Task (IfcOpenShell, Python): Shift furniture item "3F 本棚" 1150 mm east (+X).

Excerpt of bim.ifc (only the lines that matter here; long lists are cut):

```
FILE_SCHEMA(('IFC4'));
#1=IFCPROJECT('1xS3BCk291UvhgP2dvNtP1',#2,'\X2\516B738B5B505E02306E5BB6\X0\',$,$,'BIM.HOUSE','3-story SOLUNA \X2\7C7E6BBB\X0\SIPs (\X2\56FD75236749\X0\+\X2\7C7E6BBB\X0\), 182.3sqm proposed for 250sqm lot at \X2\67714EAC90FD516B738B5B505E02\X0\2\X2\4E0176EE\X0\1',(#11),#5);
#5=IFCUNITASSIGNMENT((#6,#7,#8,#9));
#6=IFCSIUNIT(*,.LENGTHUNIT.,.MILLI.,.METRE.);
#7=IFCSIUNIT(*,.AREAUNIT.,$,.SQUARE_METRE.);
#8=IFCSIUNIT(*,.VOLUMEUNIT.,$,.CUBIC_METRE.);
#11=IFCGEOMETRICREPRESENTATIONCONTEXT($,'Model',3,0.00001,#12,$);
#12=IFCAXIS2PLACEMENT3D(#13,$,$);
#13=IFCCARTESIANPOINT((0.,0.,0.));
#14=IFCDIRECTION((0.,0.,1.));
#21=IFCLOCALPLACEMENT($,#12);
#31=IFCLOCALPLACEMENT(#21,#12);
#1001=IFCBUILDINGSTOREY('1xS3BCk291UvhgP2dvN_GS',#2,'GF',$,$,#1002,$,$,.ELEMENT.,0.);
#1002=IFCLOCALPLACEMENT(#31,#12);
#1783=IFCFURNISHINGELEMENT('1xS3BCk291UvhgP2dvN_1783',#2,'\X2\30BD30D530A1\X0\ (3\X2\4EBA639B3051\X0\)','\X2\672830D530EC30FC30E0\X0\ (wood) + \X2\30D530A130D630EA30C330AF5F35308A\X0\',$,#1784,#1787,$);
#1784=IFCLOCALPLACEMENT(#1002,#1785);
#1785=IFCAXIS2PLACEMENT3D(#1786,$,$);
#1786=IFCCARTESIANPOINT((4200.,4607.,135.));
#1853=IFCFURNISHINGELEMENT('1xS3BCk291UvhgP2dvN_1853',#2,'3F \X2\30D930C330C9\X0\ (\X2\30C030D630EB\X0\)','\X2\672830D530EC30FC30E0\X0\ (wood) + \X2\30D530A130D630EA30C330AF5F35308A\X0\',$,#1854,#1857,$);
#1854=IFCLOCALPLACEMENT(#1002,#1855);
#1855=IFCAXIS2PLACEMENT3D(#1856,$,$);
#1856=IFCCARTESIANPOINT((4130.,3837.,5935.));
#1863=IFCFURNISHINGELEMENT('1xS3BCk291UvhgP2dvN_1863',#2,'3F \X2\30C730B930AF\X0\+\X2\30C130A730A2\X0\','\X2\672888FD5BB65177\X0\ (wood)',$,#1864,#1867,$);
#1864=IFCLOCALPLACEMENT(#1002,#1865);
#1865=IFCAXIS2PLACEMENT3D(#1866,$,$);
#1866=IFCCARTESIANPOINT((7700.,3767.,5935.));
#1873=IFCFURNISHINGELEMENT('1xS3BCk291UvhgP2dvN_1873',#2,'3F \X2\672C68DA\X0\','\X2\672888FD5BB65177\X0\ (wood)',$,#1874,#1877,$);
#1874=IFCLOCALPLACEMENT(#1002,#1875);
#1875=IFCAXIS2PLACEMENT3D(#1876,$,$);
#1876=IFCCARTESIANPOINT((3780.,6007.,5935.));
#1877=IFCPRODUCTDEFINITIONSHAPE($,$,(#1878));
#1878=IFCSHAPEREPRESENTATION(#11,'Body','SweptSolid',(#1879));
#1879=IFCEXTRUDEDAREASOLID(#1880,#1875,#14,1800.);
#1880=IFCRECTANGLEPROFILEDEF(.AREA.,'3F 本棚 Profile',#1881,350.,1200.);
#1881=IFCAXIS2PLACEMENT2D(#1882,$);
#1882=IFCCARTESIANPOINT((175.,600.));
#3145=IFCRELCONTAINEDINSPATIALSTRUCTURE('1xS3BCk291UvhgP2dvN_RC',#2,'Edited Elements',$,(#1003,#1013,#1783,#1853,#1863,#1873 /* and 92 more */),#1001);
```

```python
import ifcopenshell
import ifcopenshell.api.geometry
import ifcopenshell.util.placement

model = ifcopenshell.open("bim.ifc")

item = model.by_guid("1xS3BCk291UvhgP2dvN_1873")
matrix = ifcopenshell.util.placement.get_local_placement(item.ObjectPlacement)
matrix[0, 3] += 1150.0
ifcopenshell.api.geometry.edit_object_placement(model, product=item, matrix=matrix, is_si=False)

print(ifcopenshell.util.placement.get_local_placement(item.ObjectPlacement).round(3) + 0.0)

model.write("bim_updated.ifc")
```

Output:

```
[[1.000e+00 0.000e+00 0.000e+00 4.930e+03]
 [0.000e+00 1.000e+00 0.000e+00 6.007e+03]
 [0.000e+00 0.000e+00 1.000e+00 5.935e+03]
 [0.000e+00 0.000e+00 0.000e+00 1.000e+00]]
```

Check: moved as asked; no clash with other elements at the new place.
